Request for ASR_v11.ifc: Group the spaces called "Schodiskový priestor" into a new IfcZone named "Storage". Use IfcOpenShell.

First a look at what the model holds.

```python
import ifcopenshell

model = ifcopenshell.open("ASR_v11.ifc")
print(model.schema)
seen = {}
for space in model.by_type("IfcSpace"):
    seen[space.LongName] = seen.get(space.LongName, 0) + 1
for name, count in sorted(seen.items(), key=str):
    print(count, "x", name)
print("zones:", [z.Name for z in model.by_type("IfcZone")][:20])
```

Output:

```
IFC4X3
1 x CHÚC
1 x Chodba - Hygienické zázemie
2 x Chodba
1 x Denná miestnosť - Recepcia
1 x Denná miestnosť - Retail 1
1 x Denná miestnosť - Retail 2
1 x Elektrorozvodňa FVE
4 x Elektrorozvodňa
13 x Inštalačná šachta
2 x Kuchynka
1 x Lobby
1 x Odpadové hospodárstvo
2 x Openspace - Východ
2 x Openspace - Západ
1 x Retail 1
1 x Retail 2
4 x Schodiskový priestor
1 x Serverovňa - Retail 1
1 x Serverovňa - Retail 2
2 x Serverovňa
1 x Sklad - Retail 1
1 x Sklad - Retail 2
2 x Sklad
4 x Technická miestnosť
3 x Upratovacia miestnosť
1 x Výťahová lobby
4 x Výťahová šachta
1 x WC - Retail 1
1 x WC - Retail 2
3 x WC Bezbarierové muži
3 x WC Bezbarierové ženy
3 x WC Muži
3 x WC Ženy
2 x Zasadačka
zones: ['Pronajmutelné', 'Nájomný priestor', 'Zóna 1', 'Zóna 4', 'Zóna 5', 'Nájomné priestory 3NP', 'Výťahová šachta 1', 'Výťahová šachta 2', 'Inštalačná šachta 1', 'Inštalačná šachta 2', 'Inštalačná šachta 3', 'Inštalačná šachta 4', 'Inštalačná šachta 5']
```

```python
import ifcopenshell
import ifcopenshell.api.group
import ifcopenshell.api.root

model = ifcopenshell.open("ASR_v11.ifc")

names = {"Schodiskový priestor"}
spaces = [s for s in model.by_type("IfcSpace") if s.LongName in names]

zone = ifcopenshell.api.root.create_entity(model, ifc_class="IfcZone", name="Storage")
ifcopenshell.api.group.assign_group(model, products=spaces, group=zone)
print(len(spaces), "spaces in", zone.Name)

model.write("ASR_v11_edited.ifc")
```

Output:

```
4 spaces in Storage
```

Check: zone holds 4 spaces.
